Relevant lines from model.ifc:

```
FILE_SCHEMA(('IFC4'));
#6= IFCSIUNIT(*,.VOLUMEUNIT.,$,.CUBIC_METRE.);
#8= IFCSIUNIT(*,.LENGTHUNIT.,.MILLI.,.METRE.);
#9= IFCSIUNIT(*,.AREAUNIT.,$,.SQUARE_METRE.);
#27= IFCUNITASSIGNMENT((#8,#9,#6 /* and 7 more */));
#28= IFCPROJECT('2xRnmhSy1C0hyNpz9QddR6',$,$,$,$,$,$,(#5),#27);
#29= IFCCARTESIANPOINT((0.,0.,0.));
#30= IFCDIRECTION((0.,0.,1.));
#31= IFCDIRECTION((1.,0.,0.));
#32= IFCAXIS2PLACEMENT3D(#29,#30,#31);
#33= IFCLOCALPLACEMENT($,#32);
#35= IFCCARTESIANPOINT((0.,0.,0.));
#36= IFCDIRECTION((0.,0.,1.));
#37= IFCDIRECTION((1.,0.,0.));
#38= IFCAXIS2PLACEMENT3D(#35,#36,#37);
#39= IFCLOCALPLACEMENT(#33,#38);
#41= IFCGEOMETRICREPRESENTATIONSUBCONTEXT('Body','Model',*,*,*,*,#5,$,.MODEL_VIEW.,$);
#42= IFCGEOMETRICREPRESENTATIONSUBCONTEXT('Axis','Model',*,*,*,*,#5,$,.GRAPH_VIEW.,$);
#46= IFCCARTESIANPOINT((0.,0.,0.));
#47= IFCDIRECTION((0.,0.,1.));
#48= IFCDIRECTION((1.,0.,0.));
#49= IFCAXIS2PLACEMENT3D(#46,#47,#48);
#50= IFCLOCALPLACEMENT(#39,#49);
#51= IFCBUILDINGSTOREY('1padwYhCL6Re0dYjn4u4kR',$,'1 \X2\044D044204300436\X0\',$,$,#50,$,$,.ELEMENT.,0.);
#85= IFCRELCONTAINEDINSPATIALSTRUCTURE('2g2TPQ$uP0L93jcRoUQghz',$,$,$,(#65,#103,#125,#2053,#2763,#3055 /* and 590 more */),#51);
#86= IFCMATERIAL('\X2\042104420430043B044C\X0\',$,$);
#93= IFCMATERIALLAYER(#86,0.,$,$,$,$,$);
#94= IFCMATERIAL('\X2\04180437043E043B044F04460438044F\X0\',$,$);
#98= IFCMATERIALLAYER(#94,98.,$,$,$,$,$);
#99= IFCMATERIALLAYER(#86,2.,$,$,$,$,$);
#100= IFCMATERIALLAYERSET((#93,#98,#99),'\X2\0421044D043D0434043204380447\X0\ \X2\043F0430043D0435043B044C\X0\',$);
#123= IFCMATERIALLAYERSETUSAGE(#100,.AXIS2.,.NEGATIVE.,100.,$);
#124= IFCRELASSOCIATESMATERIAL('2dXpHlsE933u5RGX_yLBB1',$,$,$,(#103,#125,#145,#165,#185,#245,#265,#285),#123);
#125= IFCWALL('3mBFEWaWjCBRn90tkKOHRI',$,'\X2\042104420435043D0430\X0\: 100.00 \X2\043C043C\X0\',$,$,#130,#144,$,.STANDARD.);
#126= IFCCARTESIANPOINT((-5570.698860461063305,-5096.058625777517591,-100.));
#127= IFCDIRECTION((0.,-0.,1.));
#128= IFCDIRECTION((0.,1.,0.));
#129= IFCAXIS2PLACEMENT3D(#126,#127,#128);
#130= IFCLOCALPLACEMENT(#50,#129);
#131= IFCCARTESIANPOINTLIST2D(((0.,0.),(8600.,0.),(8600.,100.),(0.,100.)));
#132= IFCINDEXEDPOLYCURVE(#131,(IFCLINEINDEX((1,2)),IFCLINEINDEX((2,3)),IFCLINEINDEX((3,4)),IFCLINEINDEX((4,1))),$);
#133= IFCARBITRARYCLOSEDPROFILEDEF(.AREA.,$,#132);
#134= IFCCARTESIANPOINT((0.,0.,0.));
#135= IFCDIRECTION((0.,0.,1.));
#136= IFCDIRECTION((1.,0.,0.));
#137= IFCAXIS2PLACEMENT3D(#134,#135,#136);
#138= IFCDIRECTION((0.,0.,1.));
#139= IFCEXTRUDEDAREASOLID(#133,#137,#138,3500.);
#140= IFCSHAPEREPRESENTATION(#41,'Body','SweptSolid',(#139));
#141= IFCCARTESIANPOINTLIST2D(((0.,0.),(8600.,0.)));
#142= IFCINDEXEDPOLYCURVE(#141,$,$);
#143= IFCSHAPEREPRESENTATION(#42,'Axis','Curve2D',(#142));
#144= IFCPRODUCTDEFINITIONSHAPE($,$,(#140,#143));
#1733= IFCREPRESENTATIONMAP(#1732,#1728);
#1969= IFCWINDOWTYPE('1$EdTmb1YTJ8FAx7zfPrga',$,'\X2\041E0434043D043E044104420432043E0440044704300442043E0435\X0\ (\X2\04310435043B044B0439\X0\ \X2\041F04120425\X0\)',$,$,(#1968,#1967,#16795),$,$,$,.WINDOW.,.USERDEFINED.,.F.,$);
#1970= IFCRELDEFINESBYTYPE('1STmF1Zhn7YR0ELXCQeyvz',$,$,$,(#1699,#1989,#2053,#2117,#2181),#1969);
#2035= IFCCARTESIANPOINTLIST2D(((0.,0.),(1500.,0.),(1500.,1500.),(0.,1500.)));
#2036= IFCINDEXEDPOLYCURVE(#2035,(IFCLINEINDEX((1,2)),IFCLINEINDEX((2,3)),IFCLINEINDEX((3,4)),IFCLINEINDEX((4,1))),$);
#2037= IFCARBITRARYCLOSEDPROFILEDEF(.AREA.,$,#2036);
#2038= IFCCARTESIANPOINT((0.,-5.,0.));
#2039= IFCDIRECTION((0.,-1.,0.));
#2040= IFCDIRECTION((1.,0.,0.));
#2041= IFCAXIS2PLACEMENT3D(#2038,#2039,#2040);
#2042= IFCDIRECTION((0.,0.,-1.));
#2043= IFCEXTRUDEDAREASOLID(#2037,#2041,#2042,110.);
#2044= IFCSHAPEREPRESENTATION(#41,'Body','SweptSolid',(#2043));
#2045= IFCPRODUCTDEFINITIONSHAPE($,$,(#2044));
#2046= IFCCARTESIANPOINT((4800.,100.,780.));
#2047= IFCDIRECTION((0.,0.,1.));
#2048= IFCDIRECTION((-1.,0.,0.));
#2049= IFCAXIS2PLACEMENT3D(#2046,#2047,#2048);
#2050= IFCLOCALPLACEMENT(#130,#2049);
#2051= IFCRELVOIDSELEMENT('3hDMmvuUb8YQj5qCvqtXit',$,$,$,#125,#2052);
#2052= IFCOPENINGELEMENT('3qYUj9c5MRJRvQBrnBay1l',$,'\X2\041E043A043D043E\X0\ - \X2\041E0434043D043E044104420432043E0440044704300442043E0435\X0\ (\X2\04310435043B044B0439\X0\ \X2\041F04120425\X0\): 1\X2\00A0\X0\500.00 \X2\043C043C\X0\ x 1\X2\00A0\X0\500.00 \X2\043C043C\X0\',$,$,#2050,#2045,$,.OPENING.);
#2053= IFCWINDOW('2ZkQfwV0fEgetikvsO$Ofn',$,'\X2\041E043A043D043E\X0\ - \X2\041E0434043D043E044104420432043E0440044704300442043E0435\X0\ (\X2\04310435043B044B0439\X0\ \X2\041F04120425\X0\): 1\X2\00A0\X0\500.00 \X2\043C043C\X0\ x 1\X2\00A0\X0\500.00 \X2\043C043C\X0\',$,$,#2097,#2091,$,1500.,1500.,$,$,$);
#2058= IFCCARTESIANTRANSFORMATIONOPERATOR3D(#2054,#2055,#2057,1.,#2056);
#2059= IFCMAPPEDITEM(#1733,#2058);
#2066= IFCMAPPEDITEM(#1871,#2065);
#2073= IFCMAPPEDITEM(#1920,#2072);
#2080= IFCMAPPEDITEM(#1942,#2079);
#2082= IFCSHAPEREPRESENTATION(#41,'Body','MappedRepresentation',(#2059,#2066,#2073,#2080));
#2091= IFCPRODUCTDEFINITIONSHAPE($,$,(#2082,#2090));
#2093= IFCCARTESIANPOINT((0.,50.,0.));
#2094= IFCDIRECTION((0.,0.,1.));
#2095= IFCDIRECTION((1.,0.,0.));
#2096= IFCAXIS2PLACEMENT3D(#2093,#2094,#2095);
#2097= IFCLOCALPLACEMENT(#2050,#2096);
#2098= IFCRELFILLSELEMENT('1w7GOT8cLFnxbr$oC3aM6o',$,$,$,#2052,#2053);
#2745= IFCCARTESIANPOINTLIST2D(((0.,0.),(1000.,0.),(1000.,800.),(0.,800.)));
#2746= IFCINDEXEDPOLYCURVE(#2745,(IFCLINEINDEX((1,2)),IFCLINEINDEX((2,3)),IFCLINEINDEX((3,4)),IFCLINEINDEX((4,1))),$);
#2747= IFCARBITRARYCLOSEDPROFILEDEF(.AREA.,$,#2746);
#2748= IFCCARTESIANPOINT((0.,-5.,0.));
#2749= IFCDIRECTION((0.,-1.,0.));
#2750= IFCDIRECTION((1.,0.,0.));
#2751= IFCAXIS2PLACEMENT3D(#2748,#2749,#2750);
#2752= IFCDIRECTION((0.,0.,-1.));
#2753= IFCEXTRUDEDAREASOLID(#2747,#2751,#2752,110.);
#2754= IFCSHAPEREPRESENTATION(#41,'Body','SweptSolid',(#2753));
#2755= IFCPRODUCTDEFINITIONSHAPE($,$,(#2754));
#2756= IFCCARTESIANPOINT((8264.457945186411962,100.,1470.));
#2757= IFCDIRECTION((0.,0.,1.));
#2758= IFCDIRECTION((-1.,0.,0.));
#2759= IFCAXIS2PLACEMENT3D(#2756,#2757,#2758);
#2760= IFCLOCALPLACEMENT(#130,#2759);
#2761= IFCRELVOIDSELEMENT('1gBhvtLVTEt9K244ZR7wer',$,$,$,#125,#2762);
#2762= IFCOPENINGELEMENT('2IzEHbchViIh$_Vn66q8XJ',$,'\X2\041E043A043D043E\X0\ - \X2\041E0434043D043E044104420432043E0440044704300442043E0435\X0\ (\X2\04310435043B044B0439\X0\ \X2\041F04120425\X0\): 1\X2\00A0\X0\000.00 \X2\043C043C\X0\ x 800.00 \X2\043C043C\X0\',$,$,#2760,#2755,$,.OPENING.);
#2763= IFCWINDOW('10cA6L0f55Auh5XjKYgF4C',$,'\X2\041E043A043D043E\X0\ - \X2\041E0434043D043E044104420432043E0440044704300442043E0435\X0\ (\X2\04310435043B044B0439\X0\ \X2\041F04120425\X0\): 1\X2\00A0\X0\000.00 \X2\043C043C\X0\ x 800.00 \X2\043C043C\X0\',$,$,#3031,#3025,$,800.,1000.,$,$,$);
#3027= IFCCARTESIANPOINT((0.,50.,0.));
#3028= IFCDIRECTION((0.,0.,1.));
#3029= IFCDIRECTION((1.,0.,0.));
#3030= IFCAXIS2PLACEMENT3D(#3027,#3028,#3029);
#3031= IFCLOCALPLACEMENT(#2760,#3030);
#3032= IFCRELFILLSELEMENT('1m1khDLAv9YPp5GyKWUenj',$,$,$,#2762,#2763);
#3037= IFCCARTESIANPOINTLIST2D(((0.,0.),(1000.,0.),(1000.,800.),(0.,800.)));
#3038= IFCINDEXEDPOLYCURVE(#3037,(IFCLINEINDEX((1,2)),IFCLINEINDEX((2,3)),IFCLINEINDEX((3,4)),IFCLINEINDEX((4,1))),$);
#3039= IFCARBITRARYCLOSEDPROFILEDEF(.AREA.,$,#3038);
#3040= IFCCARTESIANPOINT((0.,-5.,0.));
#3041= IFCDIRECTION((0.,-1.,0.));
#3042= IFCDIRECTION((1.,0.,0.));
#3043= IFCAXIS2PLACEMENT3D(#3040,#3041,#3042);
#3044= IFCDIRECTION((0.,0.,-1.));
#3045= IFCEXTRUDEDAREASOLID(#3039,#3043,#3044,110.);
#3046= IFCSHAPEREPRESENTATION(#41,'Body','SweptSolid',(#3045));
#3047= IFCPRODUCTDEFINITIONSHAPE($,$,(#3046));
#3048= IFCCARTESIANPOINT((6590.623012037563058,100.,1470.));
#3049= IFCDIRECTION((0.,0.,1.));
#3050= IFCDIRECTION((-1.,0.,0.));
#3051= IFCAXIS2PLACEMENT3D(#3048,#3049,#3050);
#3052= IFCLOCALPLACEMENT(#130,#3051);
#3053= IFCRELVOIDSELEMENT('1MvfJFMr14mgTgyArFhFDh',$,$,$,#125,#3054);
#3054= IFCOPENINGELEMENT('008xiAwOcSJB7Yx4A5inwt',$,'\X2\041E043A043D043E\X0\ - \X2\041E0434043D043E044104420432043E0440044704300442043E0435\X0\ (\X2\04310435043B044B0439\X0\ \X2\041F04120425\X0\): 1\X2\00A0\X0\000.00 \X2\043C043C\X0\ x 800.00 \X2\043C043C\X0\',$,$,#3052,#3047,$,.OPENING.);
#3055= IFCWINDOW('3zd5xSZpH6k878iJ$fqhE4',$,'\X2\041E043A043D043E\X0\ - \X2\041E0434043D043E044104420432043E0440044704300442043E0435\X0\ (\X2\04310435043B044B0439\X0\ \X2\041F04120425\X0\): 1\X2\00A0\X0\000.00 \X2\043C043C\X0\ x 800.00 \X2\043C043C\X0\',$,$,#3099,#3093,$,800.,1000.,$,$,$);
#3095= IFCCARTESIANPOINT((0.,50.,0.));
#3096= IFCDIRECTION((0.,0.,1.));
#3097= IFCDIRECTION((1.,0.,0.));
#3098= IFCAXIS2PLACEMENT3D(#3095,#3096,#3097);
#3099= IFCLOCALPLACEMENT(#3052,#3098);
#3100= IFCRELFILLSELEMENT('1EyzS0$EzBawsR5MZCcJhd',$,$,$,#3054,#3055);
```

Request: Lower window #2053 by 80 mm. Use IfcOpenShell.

```python
import numpy as np
import ifcopenshell
import ifcopenshell.api.geometry
import ifcopenshell.util.placement
import ifcopenshell.util.unit

model = ifcopenshell.open("model.ifc")
unit_scale = ifcopenshell.util.unit.calculate_unit_scale(model)

window = model.by_guid("2ZkQfwV0fEgetikvsO$Ofn")
opening = window.FillsVoids[0].RelatingOpeningElement
dz = -0.08 / unit_scale

shift = np.array([0.0, 0.0, dz])
# The window is placed relative to its opening, so it follows when the opening moves.
matrix = ifcopenshell.util.placement.get_local_placement(opening.ObjectPlacement)
matrix[:3, 3] += shift
ifcopenshell.api.geometry.edit_object_placement(
    model, product=opening, matrix=matrix, is_si=False, should_transform_children=True
)

print(f"moved by {dz * unit_scale:+.3f} m")

model.write("model-out.ifc")
```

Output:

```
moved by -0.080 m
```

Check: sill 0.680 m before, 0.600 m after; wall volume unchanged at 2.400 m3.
